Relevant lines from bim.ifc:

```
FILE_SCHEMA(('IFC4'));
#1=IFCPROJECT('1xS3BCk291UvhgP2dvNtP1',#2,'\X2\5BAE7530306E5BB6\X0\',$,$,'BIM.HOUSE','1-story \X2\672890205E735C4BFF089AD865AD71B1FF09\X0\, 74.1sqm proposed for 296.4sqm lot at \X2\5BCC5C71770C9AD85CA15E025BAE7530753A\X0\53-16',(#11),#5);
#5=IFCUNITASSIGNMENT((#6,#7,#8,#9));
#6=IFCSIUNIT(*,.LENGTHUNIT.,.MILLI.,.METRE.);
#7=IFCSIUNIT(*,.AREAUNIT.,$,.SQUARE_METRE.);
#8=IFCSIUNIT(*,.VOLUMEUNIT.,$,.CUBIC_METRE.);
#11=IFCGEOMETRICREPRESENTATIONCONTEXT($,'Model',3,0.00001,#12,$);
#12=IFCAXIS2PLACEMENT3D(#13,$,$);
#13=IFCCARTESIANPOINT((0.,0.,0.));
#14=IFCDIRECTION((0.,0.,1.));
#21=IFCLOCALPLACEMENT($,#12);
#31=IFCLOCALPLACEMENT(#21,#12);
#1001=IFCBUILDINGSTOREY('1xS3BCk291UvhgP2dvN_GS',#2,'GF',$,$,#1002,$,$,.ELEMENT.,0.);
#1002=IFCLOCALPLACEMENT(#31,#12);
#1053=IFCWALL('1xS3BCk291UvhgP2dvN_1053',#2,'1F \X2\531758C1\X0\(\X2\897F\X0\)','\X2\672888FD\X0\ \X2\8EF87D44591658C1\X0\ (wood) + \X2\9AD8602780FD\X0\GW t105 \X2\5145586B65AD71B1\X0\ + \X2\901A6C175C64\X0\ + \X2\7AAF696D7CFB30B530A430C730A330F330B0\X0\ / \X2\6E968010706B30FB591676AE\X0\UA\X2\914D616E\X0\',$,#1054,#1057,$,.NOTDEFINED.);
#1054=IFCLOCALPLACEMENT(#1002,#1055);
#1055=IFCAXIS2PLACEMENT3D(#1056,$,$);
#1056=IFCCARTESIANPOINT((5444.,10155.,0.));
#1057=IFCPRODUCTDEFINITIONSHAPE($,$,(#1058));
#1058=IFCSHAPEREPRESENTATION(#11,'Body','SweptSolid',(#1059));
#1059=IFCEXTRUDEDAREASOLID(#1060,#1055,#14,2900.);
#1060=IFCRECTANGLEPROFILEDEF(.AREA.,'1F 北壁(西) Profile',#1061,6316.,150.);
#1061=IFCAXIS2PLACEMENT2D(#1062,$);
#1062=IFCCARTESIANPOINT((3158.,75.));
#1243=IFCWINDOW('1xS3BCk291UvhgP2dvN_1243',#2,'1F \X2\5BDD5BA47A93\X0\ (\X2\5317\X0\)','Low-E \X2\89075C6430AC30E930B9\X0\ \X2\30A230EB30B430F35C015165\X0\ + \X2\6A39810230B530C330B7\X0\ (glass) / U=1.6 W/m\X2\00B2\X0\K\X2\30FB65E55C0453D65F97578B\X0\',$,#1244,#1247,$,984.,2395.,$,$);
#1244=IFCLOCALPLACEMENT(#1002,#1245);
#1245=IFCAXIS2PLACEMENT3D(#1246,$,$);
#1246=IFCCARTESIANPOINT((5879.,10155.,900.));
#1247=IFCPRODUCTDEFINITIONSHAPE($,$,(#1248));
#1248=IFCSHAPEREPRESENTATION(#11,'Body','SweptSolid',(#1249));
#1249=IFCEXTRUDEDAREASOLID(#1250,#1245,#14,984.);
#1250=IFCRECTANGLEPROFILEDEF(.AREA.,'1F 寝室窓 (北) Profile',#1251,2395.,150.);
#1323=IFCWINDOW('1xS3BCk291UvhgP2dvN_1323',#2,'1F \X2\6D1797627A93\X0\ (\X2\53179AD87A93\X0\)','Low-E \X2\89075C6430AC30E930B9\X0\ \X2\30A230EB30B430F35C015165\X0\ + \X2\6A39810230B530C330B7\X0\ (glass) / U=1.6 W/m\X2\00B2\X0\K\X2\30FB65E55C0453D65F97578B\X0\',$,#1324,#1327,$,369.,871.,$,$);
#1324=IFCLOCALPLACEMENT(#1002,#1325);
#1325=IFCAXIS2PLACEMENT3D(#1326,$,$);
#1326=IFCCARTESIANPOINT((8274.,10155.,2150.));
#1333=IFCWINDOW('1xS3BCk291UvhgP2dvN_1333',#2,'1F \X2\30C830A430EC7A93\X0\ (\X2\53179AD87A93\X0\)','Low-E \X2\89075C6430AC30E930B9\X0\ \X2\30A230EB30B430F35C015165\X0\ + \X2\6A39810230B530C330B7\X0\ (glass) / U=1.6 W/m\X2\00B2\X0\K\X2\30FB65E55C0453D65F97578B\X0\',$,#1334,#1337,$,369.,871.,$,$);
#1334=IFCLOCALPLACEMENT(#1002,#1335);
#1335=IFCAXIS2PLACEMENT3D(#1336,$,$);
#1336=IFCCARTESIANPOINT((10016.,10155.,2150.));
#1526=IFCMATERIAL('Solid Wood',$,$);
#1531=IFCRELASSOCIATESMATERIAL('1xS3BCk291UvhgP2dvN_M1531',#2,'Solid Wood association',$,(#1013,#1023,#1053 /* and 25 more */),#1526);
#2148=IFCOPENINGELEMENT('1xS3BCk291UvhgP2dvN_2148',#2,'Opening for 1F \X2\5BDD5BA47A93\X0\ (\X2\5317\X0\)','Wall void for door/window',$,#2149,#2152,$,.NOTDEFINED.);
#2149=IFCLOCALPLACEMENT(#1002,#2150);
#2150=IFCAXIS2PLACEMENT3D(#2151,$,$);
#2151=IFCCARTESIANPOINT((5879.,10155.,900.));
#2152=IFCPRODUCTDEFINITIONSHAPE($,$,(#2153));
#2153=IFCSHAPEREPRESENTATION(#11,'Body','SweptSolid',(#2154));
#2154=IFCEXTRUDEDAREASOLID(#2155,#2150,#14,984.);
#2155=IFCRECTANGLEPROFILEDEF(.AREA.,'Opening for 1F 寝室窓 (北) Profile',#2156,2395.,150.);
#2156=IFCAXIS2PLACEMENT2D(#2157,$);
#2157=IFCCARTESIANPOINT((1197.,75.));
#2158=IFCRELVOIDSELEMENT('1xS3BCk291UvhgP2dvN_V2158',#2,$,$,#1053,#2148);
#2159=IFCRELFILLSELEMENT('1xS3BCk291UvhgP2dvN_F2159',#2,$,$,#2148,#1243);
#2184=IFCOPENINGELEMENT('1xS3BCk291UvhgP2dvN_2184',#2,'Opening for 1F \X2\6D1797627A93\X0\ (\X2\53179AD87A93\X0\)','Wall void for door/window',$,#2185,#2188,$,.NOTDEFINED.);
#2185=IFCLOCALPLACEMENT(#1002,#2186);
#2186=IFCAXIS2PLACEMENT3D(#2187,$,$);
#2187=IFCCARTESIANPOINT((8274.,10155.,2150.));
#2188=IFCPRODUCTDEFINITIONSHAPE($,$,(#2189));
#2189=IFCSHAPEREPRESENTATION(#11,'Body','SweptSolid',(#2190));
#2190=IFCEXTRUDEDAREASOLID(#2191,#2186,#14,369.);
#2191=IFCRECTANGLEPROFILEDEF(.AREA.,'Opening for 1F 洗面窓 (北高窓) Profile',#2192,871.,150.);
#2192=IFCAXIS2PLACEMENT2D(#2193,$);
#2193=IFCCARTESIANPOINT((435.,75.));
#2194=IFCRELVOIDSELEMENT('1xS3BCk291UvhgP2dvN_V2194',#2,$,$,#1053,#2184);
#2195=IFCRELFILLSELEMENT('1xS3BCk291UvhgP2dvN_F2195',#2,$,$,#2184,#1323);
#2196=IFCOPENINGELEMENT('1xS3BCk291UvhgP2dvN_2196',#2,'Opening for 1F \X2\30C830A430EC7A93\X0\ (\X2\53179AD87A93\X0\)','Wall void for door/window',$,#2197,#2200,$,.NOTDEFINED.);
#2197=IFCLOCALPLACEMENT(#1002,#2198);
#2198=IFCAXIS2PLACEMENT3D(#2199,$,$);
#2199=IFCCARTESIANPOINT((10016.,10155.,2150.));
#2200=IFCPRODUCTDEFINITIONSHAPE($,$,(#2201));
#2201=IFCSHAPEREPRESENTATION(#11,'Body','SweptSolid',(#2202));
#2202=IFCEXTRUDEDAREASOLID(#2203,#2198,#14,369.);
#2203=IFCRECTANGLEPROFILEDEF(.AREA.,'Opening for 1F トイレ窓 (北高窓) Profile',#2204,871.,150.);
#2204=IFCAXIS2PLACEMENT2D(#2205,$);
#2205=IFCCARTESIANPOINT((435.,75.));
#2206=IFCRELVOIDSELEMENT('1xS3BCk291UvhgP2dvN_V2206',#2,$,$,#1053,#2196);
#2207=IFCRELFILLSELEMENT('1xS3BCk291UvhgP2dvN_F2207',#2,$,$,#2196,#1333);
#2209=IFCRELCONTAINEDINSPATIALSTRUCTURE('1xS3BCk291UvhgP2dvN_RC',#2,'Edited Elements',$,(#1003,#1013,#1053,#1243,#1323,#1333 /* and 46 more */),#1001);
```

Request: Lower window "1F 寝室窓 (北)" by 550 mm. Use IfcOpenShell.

```python
import numpy as np
import ifcopenshell
import ifcopenshell.api.geometry
import ifcopenshell.util.placement
import ifcopenshell.util.unit

model = ifcopenshell.open("bim.ifc")
unit_scale = ifcopenshell.util.unit.calculate_unit_scale(model)

window = model.by_id(1243)
opening = window.FillsVoids[0].RelatingOpeningElement
dz = -0.55 / unit_scale

shift = np.array([0.0, 0.0, dz])
# The window is not placed relative to its opening, so move both.
for product in (opening, window):
    matrix = ifcopenshell.util.placement.get_local_placement(product.ObjectPlacement)
    matrix[:3, 3] += shift
    ifcopenshell.api.geometry.edit_object_placement(model, product=product, matrix=matrix, is_si=False)

print(f"moved by {dz * unit_scale:+.3f} m")

model.write("bim_rev.ifc")
```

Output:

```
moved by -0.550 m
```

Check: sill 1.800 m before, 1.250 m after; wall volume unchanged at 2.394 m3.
